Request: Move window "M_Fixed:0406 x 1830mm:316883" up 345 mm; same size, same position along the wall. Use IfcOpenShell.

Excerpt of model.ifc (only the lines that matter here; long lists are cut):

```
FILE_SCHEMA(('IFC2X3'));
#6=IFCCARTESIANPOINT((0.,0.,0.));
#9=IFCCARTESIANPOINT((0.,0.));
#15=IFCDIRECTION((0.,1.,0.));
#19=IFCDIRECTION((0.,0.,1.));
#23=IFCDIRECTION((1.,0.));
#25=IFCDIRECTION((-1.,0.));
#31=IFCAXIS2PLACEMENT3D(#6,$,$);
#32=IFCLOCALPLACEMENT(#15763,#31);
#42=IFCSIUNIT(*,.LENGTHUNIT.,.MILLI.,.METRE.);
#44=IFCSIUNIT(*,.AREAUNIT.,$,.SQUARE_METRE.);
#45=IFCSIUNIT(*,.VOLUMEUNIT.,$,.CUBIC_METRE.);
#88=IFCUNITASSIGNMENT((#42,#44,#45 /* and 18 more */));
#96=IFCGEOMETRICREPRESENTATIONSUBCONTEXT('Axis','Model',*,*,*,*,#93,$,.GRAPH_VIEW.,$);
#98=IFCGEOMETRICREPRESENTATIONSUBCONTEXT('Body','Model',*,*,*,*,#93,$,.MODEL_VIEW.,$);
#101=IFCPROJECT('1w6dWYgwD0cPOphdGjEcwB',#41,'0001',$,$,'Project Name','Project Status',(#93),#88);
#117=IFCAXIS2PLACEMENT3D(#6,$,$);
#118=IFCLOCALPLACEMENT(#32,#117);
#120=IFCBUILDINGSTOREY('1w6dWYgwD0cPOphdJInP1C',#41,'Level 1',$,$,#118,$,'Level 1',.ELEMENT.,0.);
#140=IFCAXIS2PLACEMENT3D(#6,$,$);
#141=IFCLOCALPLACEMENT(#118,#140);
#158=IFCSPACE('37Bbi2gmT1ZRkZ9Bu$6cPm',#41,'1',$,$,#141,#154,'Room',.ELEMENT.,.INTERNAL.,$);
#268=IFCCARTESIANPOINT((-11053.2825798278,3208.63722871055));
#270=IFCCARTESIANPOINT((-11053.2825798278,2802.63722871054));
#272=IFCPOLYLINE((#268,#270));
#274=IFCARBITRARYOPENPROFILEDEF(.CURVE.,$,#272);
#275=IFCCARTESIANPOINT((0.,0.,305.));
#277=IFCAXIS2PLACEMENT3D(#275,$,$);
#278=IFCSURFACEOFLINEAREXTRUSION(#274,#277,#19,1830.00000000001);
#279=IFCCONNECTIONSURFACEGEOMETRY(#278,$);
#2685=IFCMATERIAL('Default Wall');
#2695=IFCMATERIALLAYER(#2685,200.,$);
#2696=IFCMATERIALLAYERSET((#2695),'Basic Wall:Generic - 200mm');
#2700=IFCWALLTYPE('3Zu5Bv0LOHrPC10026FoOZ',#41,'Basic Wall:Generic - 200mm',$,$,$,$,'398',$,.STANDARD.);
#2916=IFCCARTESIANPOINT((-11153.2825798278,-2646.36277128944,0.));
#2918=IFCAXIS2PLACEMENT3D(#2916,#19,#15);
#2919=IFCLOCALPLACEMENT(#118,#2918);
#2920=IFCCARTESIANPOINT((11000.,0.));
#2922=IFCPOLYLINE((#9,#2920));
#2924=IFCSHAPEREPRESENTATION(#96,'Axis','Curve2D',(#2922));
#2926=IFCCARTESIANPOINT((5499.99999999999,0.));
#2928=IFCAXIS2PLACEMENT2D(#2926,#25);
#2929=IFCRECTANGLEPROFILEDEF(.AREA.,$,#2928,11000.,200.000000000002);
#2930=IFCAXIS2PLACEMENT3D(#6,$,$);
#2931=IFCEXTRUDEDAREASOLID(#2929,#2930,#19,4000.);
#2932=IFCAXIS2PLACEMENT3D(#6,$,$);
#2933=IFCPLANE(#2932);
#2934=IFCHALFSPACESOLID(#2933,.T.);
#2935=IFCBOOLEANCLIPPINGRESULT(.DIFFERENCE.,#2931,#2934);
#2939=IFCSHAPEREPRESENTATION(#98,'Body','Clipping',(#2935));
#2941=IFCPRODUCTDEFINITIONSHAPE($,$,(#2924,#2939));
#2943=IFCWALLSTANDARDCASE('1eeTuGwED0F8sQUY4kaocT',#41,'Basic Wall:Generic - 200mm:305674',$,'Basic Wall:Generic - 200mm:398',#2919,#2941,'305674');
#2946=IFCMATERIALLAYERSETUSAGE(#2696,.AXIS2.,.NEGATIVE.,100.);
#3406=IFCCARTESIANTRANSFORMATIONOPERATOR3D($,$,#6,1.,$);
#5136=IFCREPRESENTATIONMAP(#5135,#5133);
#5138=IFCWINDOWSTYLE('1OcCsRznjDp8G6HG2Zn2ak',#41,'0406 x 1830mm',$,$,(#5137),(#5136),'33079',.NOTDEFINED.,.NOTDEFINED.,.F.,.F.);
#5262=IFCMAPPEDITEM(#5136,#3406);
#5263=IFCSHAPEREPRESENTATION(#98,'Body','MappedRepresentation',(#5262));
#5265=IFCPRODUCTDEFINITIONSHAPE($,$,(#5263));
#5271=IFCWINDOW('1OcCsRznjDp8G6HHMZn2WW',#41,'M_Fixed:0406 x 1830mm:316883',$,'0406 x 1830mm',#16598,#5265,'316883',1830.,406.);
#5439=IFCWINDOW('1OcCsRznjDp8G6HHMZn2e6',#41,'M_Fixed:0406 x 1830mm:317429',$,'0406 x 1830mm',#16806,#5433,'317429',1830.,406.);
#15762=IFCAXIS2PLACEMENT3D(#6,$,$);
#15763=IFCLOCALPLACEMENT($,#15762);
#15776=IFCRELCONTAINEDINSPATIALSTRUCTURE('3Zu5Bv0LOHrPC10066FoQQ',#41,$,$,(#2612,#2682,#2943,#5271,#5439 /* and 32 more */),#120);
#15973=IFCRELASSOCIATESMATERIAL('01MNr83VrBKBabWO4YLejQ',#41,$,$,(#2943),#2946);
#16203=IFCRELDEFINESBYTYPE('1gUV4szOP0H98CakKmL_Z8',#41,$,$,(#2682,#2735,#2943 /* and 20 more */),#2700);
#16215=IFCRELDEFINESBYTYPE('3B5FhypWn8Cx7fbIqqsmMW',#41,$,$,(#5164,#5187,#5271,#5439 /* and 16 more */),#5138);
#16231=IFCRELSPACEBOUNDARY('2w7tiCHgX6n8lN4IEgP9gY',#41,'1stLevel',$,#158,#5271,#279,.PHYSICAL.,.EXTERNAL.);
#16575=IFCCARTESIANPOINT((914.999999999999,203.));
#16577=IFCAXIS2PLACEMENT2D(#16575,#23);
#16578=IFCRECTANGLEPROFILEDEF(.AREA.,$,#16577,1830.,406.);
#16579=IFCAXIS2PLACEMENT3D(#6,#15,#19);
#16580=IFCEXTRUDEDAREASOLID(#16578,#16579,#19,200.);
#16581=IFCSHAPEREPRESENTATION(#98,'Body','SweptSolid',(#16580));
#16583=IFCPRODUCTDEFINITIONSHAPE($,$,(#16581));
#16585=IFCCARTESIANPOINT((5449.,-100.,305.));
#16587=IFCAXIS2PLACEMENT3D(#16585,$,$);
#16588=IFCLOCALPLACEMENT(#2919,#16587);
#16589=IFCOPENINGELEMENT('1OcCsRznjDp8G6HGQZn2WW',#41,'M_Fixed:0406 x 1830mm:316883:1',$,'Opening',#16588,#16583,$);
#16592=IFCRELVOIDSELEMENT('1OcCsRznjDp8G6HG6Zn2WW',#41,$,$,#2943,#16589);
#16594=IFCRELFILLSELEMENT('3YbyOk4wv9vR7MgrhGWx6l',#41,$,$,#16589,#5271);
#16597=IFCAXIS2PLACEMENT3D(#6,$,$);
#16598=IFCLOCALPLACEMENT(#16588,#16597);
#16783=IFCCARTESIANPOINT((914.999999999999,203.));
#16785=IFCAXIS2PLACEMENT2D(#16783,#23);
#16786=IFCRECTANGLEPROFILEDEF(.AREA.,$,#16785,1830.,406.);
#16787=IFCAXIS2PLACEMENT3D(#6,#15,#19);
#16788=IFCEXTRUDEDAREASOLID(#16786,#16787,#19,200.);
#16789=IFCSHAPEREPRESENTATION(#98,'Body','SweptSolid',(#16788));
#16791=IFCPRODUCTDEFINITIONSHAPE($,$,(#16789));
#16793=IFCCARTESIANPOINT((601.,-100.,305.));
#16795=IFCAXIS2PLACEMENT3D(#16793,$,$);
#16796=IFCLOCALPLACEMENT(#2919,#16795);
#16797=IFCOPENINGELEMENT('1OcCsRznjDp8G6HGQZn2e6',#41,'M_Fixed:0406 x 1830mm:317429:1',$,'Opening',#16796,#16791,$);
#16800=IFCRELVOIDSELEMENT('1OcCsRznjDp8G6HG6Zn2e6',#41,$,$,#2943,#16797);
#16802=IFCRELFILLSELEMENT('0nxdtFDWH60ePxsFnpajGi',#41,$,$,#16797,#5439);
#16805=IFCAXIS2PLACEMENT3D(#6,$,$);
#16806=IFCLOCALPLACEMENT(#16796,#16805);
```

```python
import numpy as np
import ifcopenshell
import ifcopenshell.api.geometry
import ifcopenshell.util.placement
import ifcopenshell.util.unit

model = ifcopenshell.open("model.ifc")
unit_scale = ifcopenshell.util.unit.calculate_unit_scale(model)

window = model.by_id(5271)
opening = window.FillsVoids[0].RelatingOpeningElement
dz = 0.345 / unit_scale

shift = np.array([0.0, 0.0, dz])
# The window is placed relative to its opening, so it follows when the opening moves.
matrix = ifcopenshell.util.placement.get_local_placement(opening.ObjectPlacement)
matrix[:3, 3] += shift
ifcopenshell.api.geometry.edit_object_placement(
    model, product=opening, matrix=matrix, is_si=False, should_transform_children=True
)

# Space boundary surfaces are stored in each space's coordinates; move them too.
for rel in window.ProvidesBoundaries:
    if not rel.ConnectionGeometry:
        continue
    surface = rel.ConnectionGeometry.SurfaceOnRelatingElement
    space_matrix = ifcopenshell.util.placement.get_local_placement(rel.RelatingSpace.ObjectPlacement)
    point = np.array(surface.Position.Location.Coordinates) + space_matrix[:3, :3].T @ shift
    surface.Position = model.createIfcAxis2Placement3D(
        model.createIfcCartesianPoint(point.tolist()), surface.Position.Axis, surface.Position.RefDirection
    )

print(f"moved by {dz * unit_scale:+.3f} m")

model.write("model_v2.ifc")
```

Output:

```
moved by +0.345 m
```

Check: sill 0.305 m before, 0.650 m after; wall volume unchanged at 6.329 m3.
